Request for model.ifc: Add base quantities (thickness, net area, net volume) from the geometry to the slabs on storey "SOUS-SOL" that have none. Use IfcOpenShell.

First a look at what the model holds.

```python
import ifcopenshell
import ifcopenshell.util.element
import ifcopenshell.util.unit

model = ifcopenshell.open("model.ifc")
print(model.schema)
for unit_type in ("LENGTHUNIT", "AREAUNIT", "VOLUMEUNIT"):
    print(unit_type, ifcopenshell.util.unit.calculate_unit_scale(model, unit_type))
storey = next(s for s in model.by_type("IfcBuildingStorey") if s.Name == "SOUS-SOL")
slabs = [e for e in ifcopenshell.util.element.get_decomposition(storey) if e.is_a("IfcSlab")]
for e in sorted(slabs, key=lambda e: e.id()):
    print(e.id(), e.is_a(), e.Name, list(ifcopenshell.util.element.get_psets(e, qtos_only=True)), sep=" | ")
```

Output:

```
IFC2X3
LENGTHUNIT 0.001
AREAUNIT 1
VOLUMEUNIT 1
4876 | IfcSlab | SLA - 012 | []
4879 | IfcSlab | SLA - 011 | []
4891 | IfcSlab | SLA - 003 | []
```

```python
import ifcopenshell
import ifcopenshell.api.pset
import ifcopenshell.geom
import ifcopenshell.util.element
import ifcopenshell.util.shape
import ifcopenshell.util.unit

model = ifcopenshell.open("model.ifc")
unit_scale = ifcopenshell.util.unit.calculate_unit_scale(model)
area_scale = ifcopenshell.util.unit.calculate_unit_scale(model, "AREAUNIT")
volume_scale = ifcopenshell.util.unit.calculate_unit_scale(model, "VOLUMEUNIT")
settings = ifcopenshell.geom.settings()

storey = next(s for s in model.by_type("IfcBuildingStorey") if s.Name == "SOUS-SOL")
slabs = [e for e in ifcopenshell.util.element.get_decomposition(storey) if e.is_a("IfcSlab")]

for e in sorted(slabs, key=lambda e: e.id()):
    if ifcopenshell.util.element.get_psets(e, qtos_only=True, should_inherit=False):
        continue
    # Geometry comes back in metres, in the element's own axes.
    shape = ifcopenshell.geom.create_shape(settings, e)
    values = {
        "Width": ifcopenshell.util.shape.get_z(shape.geometry) / unit_scale,
        "NetArea": ifcopenshell.util.shape.get_footprint_area(shape.geometry) / area_scale,
        "NetVolume": ifcopenshell.util.shape.get_volume(shape.geometry) / volume_scale,
    }
    qto = ifcopenshell.api.pset.add_qto(model, product=e, name="BaseQuantities")
    ifcopenshell.api.pset.edit_qto(model, qto=qto, properties=values)
    print(e.id(), {k: round(v, 3) for k, v in values.items()})

model.write("model-out.ifc")
```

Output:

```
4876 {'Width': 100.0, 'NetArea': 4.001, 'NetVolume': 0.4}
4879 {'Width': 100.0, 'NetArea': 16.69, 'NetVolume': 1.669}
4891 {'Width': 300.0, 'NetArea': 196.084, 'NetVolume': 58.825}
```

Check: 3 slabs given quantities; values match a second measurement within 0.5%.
